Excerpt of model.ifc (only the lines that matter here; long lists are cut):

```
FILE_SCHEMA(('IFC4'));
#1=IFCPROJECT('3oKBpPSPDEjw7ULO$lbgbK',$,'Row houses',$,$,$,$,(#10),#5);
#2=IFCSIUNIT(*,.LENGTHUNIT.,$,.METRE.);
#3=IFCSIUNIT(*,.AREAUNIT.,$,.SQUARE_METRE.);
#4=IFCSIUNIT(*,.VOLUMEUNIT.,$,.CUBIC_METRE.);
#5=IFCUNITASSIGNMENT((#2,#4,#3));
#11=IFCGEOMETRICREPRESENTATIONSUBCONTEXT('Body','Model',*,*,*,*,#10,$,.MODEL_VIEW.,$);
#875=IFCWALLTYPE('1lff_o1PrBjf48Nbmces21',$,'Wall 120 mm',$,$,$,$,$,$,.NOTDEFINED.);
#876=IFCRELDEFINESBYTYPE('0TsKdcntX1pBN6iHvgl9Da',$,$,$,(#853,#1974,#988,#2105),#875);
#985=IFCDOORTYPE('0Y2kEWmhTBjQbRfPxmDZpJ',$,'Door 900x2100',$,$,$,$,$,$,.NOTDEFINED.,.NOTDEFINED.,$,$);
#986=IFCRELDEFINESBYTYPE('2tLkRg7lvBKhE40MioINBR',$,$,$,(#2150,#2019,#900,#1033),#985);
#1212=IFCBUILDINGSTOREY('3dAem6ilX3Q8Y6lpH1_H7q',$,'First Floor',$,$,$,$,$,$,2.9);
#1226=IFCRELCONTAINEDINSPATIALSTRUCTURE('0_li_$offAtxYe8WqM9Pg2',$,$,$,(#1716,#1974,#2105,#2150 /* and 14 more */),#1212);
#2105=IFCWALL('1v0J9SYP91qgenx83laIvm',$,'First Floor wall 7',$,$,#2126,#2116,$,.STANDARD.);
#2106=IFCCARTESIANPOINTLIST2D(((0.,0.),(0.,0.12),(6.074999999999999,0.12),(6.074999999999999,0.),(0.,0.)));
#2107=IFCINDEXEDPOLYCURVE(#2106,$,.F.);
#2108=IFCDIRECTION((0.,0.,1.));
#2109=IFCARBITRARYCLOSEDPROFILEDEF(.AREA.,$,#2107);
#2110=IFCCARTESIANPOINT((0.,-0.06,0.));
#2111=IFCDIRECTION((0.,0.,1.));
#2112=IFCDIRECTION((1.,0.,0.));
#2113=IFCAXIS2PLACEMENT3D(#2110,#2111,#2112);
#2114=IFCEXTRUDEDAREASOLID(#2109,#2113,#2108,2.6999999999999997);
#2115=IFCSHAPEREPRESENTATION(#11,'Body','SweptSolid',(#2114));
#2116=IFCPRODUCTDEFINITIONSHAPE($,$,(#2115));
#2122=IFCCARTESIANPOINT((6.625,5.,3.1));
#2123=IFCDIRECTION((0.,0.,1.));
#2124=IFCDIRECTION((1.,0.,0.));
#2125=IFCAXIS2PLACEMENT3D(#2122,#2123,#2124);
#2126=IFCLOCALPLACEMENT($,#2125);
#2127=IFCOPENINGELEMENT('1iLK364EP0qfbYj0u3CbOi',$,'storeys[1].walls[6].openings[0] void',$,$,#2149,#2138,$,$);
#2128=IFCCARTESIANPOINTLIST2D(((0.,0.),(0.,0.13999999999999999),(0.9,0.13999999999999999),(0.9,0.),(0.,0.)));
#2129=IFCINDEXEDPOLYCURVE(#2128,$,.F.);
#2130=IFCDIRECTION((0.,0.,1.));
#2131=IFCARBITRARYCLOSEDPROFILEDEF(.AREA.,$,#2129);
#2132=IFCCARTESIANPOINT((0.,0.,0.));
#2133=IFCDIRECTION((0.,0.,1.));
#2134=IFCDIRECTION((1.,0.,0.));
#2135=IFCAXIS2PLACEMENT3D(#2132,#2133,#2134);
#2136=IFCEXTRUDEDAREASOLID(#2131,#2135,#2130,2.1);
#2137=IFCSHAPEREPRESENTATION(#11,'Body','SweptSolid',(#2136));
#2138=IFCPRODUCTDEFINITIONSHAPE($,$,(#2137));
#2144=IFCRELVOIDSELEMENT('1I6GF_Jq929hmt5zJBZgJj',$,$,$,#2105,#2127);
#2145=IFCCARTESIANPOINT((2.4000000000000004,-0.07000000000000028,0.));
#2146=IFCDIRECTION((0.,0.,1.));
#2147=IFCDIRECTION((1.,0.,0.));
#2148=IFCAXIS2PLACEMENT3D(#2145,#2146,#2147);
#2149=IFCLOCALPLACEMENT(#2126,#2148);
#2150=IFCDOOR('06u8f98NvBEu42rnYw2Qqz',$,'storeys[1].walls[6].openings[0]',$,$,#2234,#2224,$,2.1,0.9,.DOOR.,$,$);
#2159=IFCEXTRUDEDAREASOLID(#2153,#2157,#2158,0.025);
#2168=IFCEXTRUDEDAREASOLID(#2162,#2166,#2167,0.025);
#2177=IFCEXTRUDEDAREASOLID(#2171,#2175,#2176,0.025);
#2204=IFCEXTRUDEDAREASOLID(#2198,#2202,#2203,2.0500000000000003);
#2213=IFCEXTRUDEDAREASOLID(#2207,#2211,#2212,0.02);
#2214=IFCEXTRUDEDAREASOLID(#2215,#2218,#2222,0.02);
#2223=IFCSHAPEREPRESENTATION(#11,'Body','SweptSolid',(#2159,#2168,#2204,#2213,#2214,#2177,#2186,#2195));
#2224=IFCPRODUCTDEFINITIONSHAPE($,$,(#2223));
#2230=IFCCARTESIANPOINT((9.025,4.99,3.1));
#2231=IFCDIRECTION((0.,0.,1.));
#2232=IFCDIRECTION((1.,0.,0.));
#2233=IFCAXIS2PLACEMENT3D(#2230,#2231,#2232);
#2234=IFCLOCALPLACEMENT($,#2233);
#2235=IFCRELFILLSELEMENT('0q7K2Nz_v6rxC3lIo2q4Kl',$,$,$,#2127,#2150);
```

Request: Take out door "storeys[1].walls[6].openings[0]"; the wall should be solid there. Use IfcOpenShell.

```python
import ifcopenshell
import ifcopenshell.api.feature
import ifcopenshell.api.root
import ifcopenshell.geom
import ifcopenshell.util.shape

model = ifcopenshell.open("model.ifc")
settings = ifcopenshell.geom.settings()


def volume(element):
    """Net volume in cubic metres, openings subtracted."""
    shape = ifcopenshell.geom.create_shape(settings, element)
    return ifcopenshell.util.shape.get_volume(shape.geometry)


door = model.by_guid("06u8f98NvBEu42rnYw2Qqz")
opening = door.FillsVoids[0].RelatingOpeningElement
wall = opening.VoidsElements[0].RelatingBuildingElement
before = volume(wall)

ifcopenshell.api.root.remove_product(model, product=door)
ifcopenshell.api.feature.remove_feature(model, feature=opening)

after = volume(wall)

print(f"wall volume {before:.3f} -> {after:.3f} m3")

model.write("model_rev.ifc")
```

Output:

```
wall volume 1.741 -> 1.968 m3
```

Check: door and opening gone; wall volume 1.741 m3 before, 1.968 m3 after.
